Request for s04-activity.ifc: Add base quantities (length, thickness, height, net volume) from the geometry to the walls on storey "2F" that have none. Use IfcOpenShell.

First a look at what the model holds.

```python
import ifcopenshell
import ifcopenshell.util.element
import ifcopenshell.util.unit

model = ifcopenshell.open("s04-activity.ifc")
print(model.schema)
for unit_type in ("LENGTHUNIT", "AREAUNIT", "VOLUMEUNIT"):
    print(unit_type, ifcopenshell.util.unit.calculate_unit_scale(model, unit_type))
storey = next(s for s in model.by_type("IfcBuildingStorey") if s.Name == "2F")
walls = [e for e in ifcopenshell.util.element.get_decomposition(storey) if e.is_a("IfcWall")]
for e in sorted(walls, key=lambda e: e.id()):
    print(e.id(), e.is_a(), e.Name, list(ifcopenshell.util.element.get_psets(e, qtos_only=True)), sep=" | ")
```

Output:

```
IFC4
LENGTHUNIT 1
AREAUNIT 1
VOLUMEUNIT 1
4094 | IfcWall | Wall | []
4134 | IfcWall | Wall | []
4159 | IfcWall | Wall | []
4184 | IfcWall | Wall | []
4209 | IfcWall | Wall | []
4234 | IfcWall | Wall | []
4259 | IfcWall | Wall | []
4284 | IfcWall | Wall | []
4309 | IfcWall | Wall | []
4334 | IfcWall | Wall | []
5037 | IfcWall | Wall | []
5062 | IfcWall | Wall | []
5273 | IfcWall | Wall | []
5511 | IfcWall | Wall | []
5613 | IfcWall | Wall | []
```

```python
import ifcopenshell
import ifcopenshell.api.pset
import ifcopenshell.geom
import ifcopenshell.util.element
import ifcopenshell.util.shape
import ifcopenshell.util.unit

model = ifcopenshell.open("s04-activity.ifc")
unit_scale = ifcopenshell.util.unit.calculate_unit_scale(model)
volume_scale = ifcopenshell.util.unit.calculate_unit_scale(model, "VOLUMEUNIT")
settings = ifcopenshell.geom.settings()

storey = next(s for s in model.by_type("IfcBuildingStorey") if s.Name == "2F")
walls = [e for e in ifcopenshell.util.element.get_decomposition(storey) if e.is_a("IfcWall")]

for e in sorted(walls, key=lambda e: e.id()):
    if ifcopenshell.util.element.get_psets(e, qtos_only=True, should_inherit=False):
        continue
    # Geometry comes back in metres, in the element's own axes.
    shape = ifcopenshell.geom.create_shape(settings, e)
    values = {
        "Length": ifcopenshell.util.shape.get_x(shape.geometry) / unit_scale,
        "Width": ifcopenshell.util.shape.get_y(shape.geometry) / unit_scale,
        "Height": ifcopenshell.util.shape.get_z(shape.geometry) / unit_scale,
        "NetVolume": ifcopenshell.util.shape.get_volume(shape.geometry) / volume_scale,
    }
    qto = ifcopenshell.api.pset.add_qto(model, product=e, name="Qto_WallBaseQuantities")
    ifcopenshell.api.pset.edit_qto(model, qto=qto, properties=values)
    print(e.id(), {k: round(v, 3) for k, v in values.items()})

model.write("s04-activity_edited.ifc")
```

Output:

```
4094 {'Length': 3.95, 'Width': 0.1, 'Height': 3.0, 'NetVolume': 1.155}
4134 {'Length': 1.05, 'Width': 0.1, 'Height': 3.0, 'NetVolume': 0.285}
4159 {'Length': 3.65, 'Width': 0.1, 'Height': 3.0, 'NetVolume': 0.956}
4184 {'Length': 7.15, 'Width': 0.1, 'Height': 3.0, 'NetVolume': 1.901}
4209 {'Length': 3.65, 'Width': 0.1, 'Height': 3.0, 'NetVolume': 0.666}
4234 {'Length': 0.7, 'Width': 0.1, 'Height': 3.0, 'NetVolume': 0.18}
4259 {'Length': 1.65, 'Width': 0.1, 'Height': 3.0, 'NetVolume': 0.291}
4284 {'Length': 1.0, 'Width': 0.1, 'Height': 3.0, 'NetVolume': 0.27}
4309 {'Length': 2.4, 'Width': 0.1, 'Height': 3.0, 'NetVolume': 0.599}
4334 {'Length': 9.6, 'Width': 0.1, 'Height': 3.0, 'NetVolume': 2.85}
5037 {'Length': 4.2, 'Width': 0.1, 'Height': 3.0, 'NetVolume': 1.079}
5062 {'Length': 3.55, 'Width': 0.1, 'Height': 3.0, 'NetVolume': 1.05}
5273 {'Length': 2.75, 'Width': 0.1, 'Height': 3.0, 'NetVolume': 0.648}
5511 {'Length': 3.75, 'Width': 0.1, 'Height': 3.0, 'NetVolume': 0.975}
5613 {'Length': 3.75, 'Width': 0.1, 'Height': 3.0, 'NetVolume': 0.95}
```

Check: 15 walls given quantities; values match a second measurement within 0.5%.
